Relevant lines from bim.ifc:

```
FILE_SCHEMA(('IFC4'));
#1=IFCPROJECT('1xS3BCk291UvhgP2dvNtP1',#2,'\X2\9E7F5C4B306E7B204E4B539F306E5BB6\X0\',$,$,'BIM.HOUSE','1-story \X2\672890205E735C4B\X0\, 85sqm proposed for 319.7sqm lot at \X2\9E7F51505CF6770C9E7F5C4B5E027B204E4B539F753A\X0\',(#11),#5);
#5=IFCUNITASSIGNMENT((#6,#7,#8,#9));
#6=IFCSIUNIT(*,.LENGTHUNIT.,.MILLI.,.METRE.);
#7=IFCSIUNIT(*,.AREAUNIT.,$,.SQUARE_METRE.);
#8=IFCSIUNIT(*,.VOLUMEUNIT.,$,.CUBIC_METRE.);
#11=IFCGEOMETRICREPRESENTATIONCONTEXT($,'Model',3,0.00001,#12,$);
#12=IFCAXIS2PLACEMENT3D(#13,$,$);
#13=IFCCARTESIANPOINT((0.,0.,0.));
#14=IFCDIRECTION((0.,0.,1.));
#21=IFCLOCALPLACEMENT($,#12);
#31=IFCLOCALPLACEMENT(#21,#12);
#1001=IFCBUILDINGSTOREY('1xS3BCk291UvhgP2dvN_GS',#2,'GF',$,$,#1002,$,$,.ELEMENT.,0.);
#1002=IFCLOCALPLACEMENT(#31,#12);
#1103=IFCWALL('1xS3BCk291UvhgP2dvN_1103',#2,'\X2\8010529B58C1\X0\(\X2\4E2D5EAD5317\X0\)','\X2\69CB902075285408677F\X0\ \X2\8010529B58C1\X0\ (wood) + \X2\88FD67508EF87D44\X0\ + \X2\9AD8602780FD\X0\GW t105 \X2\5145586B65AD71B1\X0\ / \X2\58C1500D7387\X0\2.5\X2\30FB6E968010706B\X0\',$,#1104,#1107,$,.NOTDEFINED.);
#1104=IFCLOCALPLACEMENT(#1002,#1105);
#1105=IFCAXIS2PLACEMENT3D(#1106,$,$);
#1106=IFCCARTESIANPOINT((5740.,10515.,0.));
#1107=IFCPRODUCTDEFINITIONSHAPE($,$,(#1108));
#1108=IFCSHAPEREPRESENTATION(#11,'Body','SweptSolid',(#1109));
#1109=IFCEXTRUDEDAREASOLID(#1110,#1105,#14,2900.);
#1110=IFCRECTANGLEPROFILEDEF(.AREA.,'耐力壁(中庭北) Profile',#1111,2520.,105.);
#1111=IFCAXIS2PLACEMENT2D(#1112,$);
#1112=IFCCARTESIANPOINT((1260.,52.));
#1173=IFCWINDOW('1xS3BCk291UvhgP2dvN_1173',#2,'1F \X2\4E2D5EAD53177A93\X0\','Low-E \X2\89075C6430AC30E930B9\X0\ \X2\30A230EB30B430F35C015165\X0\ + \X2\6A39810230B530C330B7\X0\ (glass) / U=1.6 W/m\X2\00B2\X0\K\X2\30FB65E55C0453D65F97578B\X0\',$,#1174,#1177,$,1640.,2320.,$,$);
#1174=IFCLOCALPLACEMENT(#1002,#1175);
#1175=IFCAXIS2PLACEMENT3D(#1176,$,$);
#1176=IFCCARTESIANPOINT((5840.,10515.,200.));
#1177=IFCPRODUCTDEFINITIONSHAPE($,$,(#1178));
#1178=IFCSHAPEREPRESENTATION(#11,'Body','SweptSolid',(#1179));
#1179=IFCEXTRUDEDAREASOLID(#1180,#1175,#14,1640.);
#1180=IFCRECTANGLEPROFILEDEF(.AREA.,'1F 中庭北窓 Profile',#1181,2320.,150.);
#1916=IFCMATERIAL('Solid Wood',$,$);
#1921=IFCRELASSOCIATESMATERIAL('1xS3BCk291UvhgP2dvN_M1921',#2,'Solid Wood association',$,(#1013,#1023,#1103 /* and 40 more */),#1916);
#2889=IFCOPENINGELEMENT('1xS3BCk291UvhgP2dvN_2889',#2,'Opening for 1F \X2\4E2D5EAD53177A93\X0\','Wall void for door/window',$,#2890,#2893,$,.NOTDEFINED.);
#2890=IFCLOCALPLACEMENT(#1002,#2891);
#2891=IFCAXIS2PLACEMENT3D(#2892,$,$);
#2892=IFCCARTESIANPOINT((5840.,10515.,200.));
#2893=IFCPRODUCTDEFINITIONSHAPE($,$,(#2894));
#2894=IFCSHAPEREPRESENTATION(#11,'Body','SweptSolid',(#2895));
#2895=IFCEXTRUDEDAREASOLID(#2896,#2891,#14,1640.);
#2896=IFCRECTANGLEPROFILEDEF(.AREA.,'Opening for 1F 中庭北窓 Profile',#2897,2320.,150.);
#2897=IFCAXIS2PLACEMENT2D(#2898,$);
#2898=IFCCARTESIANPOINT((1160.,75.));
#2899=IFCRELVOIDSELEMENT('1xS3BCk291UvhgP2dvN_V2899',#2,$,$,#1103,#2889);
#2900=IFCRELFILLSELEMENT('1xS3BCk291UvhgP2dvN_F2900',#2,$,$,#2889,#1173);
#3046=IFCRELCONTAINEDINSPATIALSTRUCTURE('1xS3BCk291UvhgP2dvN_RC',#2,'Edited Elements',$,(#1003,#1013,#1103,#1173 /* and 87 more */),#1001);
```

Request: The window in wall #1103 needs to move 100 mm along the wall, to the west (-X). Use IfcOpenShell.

```python
import ifcopenshell
import ifcopenshell.api.geometry
import ifcopenshell.util.placement
import ifcopenshell.util.unit

model = ifcopenshell.open("bim.ifc")
unit_scale = ifcopenshell.util.unit.calculate_unit_scale(model)

window = model.by_guid("1xS3BCk291UvhgP2dvN_1173")
opening = window.FillsVoids[0].RelatingOpeningElement
wall = opening.VoidsElements[0].RelatingBuildingElement

wall_matrix = ifcopenshell.util.placement.get_local_placement(wall.ObjectPlacement)
shift = wall_matrix[:3, 0] * -0.1 / unit_scale
before = ifcopenshell.util.placement.get_local_placement(window.ObjectPlacement)[:3, 3].copy()

# The window is not placed relative to its opening, so move both.
for product in (opening, window):
    matrix = ifcopenshell.util.placement.get_local_placement(product.ObjectPlacement)
    matrix[:3, 3] += shift
    ifcopenshell.api.geometry.edit_object_placement(model, product=product, matrix=matrix, is_si=False)

after = ifcopenshell.util.placement.get_local_placement(window.ObjectPlacement)[:3, 3]
print("window moved by", (after - before).round(3) + 0.0)

model.write("bim_rev.ifc")
```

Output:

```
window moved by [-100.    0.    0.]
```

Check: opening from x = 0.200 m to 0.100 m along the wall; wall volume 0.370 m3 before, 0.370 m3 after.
